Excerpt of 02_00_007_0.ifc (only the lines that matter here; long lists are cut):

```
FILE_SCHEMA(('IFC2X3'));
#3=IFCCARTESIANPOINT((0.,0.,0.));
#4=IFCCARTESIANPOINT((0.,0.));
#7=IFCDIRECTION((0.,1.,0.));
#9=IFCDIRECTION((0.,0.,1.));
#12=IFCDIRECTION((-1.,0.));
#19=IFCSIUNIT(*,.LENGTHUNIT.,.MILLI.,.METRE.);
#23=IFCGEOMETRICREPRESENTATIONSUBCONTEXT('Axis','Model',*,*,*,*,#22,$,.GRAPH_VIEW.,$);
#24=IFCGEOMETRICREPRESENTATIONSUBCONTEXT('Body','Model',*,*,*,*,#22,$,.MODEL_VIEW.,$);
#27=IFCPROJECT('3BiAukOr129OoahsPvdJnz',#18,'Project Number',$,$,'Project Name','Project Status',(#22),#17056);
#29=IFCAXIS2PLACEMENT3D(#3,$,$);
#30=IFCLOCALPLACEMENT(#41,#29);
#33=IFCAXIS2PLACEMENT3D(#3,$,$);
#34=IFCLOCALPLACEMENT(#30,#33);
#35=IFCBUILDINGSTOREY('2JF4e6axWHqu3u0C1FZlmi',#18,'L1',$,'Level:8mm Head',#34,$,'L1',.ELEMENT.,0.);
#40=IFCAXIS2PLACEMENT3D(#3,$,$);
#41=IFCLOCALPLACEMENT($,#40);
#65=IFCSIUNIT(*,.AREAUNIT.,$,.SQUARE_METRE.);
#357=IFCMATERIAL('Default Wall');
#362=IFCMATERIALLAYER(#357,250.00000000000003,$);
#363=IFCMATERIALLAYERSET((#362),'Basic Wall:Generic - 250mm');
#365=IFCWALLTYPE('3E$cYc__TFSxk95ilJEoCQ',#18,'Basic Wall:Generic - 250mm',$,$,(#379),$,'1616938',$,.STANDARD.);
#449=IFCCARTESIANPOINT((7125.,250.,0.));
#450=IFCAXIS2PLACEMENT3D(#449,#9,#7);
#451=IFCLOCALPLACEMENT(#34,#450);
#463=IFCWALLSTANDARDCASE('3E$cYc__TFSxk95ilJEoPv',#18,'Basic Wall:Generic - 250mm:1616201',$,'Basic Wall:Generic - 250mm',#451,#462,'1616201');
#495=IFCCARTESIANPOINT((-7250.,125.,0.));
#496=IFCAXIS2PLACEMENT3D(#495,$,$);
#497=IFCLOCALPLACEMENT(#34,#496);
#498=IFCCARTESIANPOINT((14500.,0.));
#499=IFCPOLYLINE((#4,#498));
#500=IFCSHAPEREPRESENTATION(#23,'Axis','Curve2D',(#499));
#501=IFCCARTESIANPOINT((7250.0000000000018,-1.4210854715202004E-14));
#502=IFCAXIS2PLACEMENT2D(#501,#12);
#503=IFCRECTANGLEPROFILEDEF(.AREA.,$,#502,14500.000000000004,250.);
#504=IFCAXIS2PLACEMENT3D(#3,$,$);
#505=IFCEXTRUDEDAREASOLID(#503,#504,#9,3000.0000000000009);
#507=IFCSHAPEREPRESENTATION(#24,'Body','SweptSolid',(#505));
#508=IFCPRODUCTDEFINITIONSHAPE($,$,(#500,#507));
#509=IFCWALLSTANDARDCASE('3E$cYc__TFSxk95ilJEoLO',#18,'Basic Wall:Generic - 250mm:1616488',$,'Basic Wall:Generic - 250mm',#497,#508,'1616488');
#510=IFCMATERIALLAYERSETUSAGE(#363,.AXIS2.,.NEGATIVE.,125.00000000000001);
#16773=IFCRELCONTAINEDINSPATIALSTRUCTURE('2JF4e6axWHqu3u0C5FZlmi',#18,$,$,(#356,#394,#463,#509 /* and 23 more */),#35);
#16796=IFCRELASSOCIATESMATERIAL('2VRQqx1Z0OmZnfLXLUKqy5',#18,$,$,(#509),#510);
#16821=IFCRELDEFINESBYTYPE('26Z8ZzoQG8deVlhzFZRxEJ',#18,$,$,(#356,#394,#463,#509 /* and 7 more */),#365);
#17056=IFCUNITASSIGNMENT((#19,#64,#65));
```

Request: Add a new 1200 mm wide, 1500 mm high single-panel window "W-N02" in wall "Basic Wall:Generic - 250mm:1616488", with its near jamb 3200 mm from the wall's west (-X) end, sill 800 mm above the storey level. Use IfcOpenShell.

```python
import numpy as np
import ifcopenshell
import ifcopenshell.api.feature
import ifcopenshell.api.geometry
import ifcopenshell.api.root
import ifcopenshell.api.spatial
import ifcopenshell.api.type
import ifcopenshell.geom
import ifcopenshell.util.element
import ifcopenshell.util.placement
import ifcopenshell.util.representation
import ifcopenshell.util.shape
import ifcopenshell.util.unit

model = ifcopenshell.open("02_00_007_0.ifc")
unit_scale = ifcopenshell.util.unit.calculate_unit_scale(model)
settings = ifcopenshell.geom.settings()


def volume(element):
    """Net volume in cubic metres, openings subtracted."""
    shape = ifcopenshell.geom.create_shape(settings, element)
    return ifcopenshell.util.shape.get_volume(shape.geometry)


wall = model.by_id(509)
storey = ifcopenshell.util.element.get_container(wall, ifc_class="IfcBuildingStorey")
context = ifcopenshell.util.representation.get_context(model, "Model", "Body", "MODEL_VIEW")
before = volume(wall)

width, height, from_end, sill = 1.2, 1.5, 3.2, 0.8  # metres

# The wall runs along its own X axis, and the end named is its -X end.
wall_shape = ifcopenshell.geom.create_shape(settings, wall)
x, y, z = ifcopenshell.util.shape.get_vertices(wall_shape.geometry).T
start = x.min() + from_end
face, thickness = float(y.min()), float(y.max() - y.min())
wall_matrix = ifcopenshell.util.placement.get_local_placement(wall.ObjectPlacement)
level = ifcopenshell.util.placement.get_local_placement(storey.ObjectPlacement)[2, 3]


def in_wall(x, y):
    """Placement at x, y metres in the wall's axes, at sill height."""
    matrix = wall_matrix.copy()
    matrix[:, 3] = wall_matrix @ np.array([x / unit_scale, y / unit_scale, 0.0, 1.0])
    matrix[2, 3] = level + sill / unit_scale
    return matrix


# Opening: a box that overshoots both wall faces by 50 mm.
opening = ifcopenshell.api.root.create_entity(model, ifc_class="IfcOpeningElement")
box = ifcopenshell.api.geometry.add_wall_representation(
    model, context=context, length=width, height=height, thickness=thickness + 0.1
)
ifcopenshell.api.geometry.assign_representation(model, product=opening, representation=box)
ifcopenshell.api.geometry.edit_object_placement(model, product=opening, matrix=in_wall(start, face - 0.05), is_si=False)
ifcopenshell.api.feature.add_feature(model, feature=opening, element=wall)

window = ifcopenshell.api.root.create_entity(model, ifc_class="IfcWindow", name="W-N02")
window.OverallWidth, window.OverallHeight = width / unit_scale, height / unit_scale
body = ifcopenshell.api.geometry.add_window_representation(
    model,
    context=context,
    overall_width=window.OverallWidth,
    overall_height=window.OverallHeight,
    partition_type="SINGLE_PANEL",
)
ifcopenshell.api.geometry.assign_representation(model, product=window, representation=body)
ifcopenshell.api.spatial.assign_container(model, products=[window], relating_structure=storey)
fills = ifcopenshell.api.feature.add_filling(model, opening=opening, element=window)
fills.OwnerHistory = window.OwnerHistory  # required in IFC2X3

# IFC2X3 keeps the operation on the window style.
style = ifcopenshell.api.root.create_entity(model, ifc_class="IfcWindowStyle", name="W-N02")
style.OperationType, style.ConstructionType = "SINGLE_PANEL", "NOTDEFINED"
style.ParameterTakesPrecedence = style.Sizeable = False
ifcopenshell.api.type.assign_type(model, related_objects=[window], relating_type=style)

# Centre the window in the wall's thickness.
ifcopenshell.api.geometry.edit_object_placement(model, product=window, matrix=in_wall(start, face), is_si=False)
window_shape = ifcopenshell.geom.create_shape(settings, window)
depth = ifcopenshell.util.shape.get_vertices(window_shape.geometry)[:, 1]
offset = face + thickness / 2 - (depth.min() + depth.max()) / 2
ifcopenshell.api.geometry.edit_object_placement(model, product=window, matrix=in_wall(start, offset), is_si=False)

after = volume(wall)

print(f"wall volume {before:.3f} -> {after:.3f} m3")

model.write("02_00_007_0_updated.ifc")
```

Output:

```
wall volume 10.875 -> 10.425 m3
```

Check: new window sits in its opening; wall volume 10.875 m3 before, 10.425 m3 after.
